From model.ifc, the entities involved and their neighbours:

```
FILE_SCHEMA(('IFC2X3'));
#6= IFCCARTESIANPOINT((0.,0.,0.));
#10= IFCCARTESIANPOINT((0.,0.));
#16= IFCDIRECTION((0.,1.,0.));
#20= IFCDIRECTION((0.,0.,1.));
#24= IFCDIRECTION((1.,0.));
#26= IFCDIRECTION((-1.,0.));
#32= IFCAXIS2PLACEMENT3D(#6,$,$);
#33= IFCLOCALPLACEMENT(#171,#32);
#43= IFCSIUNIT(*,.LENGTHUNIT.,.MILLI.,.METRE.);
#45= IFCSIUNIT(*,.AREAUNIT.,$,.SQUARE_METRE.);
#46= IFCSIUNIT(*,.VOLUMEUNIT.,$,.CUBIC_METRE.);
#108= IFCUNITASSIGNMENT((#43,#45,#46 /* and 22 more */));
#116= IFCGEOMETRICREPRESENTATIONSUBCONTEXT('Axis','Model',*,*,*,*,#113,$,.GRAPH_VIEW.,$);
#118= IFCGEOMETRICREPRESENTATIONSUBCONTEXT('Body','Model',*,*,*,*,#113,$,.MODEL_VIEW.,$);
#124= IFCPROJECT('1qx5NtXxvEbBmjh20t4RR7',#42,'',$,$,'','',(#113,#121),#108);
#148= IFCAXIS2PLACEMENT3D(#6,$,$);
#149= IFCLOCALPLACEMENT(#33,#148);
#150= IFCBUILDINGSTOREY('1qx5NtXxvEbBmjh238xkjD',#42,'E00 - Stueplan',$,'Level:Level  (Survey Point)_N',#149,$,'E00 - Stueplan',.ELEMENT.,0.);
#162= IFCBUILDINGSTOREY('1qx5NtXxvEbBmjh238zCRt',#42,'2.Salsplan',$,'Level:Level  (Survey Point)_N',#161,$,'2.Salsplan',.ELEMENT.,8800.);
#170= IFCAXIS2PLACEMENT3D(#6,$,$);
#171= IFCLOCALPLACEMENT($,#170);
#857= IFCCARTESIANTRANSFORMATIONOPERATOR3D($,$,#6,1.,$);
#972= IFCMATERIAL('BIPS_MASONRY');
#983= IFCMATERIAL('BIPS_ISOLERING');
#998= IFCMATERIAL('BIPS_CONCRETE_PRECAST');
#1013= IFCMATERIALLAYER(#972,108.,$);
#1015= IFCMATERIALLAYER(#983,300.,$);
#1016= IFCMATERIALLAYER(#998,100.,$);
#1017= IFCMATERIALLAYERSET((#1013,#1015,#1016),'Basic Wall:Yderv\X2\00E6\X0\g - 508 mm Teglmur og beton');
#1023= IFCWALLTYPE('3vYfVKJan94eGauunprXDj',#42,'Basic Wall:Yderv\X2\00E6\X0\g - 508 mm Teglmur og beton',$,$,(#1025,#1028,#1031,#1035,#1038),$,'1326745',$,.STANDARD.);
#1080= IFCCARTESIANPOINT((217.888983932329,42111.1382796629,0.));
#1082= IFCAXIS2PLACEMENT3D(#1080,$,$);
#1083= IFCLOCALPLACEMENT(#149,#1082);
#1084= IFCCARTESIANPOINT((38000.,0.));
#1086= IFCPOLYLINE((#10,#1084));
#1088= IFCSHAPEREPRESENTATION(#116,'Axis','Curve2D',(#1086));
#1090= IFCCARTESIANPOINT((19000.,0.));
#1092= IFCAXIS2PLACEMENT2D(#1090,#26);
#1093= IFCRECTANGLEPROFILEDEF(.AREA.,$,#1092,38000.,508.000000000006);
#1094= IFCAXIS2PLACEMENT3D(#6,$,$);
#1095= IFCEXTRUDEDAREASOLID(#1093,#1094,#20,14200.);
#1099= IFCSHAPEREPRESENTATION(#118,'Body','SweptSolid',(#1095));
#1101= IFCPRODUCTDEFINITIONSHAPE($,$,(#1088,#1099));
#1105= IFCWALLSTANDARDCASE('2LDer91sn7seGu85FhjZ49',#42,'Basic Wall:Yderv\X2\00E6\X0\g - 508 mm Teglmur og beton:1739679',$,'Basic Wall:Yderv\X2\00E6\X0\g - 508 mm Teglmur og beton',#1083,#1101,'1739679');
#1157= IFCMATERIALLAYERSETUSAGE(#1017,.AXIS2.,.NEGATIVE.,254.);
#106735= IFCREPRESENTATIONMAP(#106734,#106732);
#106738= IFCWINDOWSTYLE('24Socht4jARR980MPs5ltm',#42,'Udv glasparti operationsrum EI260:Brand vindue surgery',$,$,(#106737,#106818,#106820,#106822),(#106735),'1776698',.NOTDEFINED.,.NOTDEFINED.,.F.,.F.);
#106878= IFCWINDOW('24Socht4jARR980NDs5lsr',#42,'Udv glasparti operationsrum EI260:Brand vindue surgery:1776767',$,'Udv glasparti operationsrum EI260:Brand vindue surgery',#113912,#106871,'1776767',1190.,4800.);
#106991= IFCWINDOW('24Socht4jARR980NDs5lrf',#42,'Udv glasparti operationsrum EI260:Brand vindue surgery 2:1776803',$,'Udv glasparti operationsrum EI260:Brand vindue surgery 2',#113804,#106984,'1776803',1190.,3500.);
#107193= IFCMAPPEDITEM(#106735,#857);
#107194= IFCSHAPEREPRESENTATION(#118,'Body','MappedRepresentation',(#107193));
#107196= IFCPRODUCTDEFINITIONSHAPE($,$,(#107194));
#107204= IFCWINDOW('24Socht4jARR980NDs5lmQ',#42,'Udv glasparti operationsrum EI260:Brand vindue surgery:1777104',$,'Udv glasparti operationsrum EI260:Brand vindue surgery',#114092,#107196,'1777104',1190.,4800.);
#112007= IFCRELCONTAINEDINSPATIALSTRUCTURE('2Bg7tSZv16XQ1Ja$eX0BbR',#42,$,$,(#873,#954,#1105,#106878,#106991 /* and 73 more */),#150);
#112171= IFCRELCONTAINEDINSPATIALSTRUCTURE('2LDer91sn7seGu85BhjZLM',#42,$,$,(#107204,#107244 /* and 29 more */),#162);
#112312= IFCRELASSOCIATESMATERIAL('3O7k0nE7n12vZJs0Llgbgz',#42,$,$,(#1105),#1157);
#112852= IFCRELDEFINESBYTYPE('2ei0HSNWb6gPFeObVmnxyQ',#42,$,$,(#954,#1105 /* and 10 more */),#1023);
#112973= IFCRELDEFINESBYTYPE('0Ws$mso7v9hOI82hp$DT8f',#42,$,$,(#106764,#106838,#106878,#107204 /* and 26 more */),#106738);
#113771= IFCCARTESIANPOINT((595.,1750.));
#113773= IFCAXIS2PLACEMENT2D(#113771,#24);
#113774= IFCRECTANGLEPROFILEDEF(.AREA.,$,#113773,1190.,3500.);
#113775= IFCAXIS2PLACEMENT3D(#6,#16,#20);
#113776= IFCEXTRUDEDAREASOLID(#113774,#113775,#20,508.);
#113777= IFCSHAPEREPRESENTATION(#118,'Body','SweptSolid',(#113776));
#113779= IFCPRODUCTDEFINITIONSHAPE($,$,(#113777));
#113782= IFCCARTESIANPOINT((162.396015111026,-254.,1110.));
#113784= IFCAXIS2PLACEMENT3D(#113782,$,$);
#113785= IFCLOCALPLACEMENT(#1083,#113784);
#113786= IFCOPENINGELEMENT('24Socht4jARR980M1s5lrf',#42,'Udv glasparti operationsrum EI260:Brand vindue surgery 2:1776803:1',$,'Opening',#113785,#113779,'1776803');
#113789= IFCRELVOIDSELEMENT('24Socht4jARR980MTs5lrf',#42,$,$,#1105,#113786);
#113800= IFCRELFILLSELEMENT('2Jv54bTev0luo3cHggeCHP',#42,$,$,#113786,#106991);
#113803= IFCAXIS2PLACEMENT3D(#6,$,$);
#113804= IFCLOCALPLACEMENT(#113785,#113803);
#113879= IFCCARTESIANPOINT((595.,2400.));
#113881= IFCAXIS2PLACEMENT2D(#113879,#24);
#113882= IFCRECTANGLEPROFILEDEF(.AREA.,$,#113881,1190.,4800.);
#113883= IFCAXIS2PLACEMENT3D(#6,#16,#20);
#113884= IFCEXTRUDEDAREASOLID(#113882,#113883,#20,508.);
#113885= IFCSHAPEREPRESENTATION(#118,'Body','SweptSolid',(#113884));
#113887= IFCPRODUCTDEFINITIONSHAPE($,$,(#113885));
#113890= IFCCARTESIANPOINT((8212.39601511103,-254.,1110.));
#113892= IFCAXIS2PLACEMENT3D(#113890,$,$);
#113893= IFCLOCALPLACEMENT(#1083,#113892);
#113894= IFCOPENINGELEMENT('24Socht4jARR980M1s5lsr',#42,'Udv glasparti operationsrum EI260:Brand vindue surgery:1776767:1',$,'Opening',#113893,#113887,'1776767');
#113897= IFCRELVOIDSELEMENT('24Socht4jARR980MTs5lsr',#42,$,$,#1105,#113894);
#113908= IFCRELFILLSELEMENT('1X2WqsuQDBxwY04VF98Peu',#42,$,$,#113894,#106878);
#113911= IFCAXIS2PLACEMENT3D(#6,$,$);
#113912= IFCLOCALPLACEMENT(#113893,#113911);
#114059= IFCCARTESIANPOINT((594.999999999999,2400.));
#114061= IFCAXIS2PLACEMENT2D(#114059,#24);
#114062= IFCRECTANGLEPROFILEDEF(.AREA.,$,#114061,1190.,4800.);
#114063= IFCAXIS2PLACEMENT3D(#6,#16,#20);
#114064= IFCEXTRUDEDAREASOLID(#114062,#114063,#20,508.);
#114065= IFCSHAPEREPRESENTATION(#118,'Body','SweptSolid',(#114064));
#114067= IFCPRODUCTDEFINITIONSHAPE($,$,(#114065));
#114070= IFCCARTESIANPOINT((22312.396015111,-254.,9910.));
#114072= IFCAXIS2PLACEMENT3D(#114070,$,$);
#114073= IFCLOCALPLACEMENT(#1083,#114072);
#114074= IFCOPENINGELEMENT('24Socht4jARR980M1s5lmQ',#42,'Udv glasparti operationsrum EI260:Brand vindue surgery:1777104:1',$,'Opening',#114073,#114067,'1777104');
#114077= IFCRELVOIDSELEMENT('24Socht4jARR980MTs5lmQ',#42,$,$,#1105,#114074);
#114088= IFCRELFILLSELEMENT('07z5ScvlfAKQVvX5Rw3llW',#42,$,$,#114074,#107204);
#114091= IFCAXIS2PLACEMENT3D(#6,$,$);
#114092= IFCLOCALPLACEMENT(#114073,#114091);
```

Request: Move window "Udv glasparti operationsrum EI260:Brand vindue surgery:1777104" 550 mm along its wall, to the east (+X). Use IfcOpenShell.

```python
import ifcopenshell
import ifcopenshell.api.geometry
import ifcopenshell.util.placement
import ifcopenshell.util.unit

model = ifcopenshell.open("model.ifc")
unit_scale = ifcopenshell.util.unit.calculate_unit_scale(model)

window = model.by_guid("24Socht4jARR980NDs5lmQ")
opening = window.FillsVoids[0].RelatingOpeningElement
wall = opening.VoidsElements[0].RelatingBuildingElement

wall_matrix = ifcopenshell.util.placement.get_local_placement(wall.ObjectPlacement)
shift = wall_matrix[:3, 0] * 0.55 / unit_scale
before = ifcopenshell.util.placement.get_local_placement(window.ObjectPlacement)[:3, 3].copy()

# The window is placed relative to its opening, so it follows when the opening moves.
matrix = ifcopenshell.util.placement.get_local_placement(opening.ObjectPlacement)
matrix[:3, 3] += shift
ifcopenshell.api.geometry.edit_object_placement(
    model, product=opening, matrix=matrix, is_si=False, should_transform_children=True
)

after = ifcopenshell.util.placement.get_local_placement(window.ObjectPlacement)[:3, 3]
print("window moved by", (after - before).round(3) + 0.0)

model.write("model_updated.ifc")
```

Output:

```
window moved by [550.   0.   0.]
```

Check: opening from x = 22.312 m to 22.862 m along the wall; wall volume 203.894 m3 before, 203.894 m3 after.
